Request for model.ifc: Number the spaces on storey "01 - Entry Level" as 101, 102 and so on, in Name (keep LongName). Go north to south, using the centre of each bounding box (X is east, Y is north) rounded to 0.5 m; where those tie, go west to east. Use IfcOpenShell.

First a look at what the model holds.

```python
import ifcopenshell
import ifcopenshell.util.element
import ifcopenshell.util.placement

model = ifcopenshell.open("model.ifc")
print(model.schema)
storey = next(s for s in model.by_type("IfcBuildingStorey") if s.Name == "01 - Entry Level")
spaces = [e for e in ifcopenshell.util.element.get_decomposition(storey) if e.is_a("IfcSpace")]
for e in sorted(spaces, key=lambda e: e.id()):
    origin = ifcopenshell.util.placement.get_local_placement(e.ObjectPlacement)[:3, 3]
    print(e.id(), e.Name, e.LongName, origin.round(2) + 0.0, sep=" | ")
```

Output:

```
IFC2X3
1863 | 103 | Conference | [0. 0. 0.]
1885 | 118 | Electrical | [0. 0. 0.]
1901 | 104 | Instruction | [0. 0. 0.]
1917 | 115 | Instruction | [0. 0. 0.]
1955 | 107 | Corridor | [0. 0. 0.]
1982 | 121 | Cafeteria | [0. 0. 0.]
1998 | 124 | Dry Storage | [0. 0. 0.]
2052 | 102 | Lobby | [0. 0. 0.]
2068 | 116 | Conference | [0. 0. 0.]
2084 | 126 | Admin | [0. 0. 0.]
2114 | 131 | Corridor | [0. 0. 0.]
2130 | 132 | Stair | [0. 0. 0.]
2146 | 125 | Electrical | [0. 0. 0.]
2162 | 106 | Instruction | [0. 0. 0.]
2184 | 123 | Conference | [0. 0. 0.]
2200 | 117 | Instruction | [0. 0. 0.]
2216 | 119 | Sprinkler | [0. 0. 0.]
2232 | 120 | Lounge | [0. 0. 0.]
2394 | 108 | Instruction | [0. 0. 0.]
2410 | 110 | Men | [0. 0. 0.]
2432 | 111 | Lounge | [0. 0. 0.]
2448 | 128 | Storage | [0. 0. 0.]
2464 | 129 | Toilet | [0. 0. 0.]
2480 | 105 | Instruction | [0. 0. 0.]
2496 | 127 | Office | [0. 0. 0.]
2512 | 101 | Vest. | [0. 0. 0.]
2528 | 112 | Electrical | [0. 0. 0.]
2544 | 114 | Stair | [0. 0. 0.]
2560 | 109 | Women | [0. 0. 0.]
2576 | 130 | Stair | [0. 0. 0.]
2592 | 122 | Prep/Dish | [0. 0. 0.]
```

```python
import ifcopenshell
import ifcopenshell.geom
import ifcopenshell.util.element
import ifcopenshell.util.shape

model = ifcopenshell.open("model.ifc")
settings = ifcopenshell.geom.settings()
settings.set("use-world-coords", True)


def centre(element):
    shape = ifcopenshell.geom.create_shape(settings, element)
    return ifcopenshell.util.shape.get_bbox_centroid(shape.geometry)


storey = next(s for s in model.by_type("IfcBuildingStorey") if s.Name == "01 - Entry Level")
spaces = [e for e in ifcopenshell.util.element.get_decomposition(storey) if e.is_a("IfcSpace")]

# Insertion points can sit at a corner or the storey origin, so sort by the geometry (in metres).
centres = {e: centre(e) for e in spaces}
spaces.sort(key=lambda e: (-round(centres[e][1] / 0.5), centres[e][0]))

for i, e in enumerate(spaces, start=1):
    number = f"1{i:02d}"
    e.Name = number
    print(e.id(), number)

model.write("model-out.ifc")
```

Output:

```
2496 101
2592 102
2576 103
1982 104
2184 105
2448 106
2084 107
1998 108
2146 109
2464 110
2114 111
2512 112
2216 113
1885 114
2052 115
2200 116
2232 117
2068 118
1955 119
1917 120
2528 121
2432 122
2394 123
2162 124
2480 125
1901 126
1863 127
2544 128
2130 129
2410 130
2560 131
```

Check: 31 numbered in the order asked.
